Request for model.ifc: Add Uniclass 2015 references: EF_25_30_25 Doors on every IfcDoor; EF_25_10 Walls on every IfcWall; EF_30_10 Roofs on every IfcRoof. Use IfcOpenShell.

First a look at what the model holds.

```python
import ifcopenshell

model = ifcopenshell.open("model.ifc")
print(model.schema)
print("classifications:", [c.Name for c in model.by_type("IfcClassification")])
for ifc_class in ("IfcDoor", "IfcRoof", "IfcStair", "IfcWall", "IfcWindow"):
    print(ifc_class, len(model.by_type(ifc_class)))
```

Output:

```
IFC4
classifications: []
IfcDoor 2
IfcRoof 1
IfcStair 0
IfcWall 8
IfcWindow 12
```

```python
import ifcopenshell
import ifcopenshell.api.classification

model = ifcopenshell.open("model.ifc")

system = ifcopenshell.api.classification.add_classification(model, classification="Uniclass 2015")

codes = {
    "IfcDoor": ("EF_25_30_25", "Doors"),
    "IfcWall": ("EF_25_10", "Walls"),
    "IfcRoof": ("EF_30_10", "Roofs"),
}
for ifc_class, (code, name) in codes.items():
    products = model.by_type(ifc_class)
    ifcopenshell.api.classification.add_reference(
        model, products=products, classification=system, identification=code, name=name
    )
    print(code, len(products))

model.write("model_v2.ifc")
```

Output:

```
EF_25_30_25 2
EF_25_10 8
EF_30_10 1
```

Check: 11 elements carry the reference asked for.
